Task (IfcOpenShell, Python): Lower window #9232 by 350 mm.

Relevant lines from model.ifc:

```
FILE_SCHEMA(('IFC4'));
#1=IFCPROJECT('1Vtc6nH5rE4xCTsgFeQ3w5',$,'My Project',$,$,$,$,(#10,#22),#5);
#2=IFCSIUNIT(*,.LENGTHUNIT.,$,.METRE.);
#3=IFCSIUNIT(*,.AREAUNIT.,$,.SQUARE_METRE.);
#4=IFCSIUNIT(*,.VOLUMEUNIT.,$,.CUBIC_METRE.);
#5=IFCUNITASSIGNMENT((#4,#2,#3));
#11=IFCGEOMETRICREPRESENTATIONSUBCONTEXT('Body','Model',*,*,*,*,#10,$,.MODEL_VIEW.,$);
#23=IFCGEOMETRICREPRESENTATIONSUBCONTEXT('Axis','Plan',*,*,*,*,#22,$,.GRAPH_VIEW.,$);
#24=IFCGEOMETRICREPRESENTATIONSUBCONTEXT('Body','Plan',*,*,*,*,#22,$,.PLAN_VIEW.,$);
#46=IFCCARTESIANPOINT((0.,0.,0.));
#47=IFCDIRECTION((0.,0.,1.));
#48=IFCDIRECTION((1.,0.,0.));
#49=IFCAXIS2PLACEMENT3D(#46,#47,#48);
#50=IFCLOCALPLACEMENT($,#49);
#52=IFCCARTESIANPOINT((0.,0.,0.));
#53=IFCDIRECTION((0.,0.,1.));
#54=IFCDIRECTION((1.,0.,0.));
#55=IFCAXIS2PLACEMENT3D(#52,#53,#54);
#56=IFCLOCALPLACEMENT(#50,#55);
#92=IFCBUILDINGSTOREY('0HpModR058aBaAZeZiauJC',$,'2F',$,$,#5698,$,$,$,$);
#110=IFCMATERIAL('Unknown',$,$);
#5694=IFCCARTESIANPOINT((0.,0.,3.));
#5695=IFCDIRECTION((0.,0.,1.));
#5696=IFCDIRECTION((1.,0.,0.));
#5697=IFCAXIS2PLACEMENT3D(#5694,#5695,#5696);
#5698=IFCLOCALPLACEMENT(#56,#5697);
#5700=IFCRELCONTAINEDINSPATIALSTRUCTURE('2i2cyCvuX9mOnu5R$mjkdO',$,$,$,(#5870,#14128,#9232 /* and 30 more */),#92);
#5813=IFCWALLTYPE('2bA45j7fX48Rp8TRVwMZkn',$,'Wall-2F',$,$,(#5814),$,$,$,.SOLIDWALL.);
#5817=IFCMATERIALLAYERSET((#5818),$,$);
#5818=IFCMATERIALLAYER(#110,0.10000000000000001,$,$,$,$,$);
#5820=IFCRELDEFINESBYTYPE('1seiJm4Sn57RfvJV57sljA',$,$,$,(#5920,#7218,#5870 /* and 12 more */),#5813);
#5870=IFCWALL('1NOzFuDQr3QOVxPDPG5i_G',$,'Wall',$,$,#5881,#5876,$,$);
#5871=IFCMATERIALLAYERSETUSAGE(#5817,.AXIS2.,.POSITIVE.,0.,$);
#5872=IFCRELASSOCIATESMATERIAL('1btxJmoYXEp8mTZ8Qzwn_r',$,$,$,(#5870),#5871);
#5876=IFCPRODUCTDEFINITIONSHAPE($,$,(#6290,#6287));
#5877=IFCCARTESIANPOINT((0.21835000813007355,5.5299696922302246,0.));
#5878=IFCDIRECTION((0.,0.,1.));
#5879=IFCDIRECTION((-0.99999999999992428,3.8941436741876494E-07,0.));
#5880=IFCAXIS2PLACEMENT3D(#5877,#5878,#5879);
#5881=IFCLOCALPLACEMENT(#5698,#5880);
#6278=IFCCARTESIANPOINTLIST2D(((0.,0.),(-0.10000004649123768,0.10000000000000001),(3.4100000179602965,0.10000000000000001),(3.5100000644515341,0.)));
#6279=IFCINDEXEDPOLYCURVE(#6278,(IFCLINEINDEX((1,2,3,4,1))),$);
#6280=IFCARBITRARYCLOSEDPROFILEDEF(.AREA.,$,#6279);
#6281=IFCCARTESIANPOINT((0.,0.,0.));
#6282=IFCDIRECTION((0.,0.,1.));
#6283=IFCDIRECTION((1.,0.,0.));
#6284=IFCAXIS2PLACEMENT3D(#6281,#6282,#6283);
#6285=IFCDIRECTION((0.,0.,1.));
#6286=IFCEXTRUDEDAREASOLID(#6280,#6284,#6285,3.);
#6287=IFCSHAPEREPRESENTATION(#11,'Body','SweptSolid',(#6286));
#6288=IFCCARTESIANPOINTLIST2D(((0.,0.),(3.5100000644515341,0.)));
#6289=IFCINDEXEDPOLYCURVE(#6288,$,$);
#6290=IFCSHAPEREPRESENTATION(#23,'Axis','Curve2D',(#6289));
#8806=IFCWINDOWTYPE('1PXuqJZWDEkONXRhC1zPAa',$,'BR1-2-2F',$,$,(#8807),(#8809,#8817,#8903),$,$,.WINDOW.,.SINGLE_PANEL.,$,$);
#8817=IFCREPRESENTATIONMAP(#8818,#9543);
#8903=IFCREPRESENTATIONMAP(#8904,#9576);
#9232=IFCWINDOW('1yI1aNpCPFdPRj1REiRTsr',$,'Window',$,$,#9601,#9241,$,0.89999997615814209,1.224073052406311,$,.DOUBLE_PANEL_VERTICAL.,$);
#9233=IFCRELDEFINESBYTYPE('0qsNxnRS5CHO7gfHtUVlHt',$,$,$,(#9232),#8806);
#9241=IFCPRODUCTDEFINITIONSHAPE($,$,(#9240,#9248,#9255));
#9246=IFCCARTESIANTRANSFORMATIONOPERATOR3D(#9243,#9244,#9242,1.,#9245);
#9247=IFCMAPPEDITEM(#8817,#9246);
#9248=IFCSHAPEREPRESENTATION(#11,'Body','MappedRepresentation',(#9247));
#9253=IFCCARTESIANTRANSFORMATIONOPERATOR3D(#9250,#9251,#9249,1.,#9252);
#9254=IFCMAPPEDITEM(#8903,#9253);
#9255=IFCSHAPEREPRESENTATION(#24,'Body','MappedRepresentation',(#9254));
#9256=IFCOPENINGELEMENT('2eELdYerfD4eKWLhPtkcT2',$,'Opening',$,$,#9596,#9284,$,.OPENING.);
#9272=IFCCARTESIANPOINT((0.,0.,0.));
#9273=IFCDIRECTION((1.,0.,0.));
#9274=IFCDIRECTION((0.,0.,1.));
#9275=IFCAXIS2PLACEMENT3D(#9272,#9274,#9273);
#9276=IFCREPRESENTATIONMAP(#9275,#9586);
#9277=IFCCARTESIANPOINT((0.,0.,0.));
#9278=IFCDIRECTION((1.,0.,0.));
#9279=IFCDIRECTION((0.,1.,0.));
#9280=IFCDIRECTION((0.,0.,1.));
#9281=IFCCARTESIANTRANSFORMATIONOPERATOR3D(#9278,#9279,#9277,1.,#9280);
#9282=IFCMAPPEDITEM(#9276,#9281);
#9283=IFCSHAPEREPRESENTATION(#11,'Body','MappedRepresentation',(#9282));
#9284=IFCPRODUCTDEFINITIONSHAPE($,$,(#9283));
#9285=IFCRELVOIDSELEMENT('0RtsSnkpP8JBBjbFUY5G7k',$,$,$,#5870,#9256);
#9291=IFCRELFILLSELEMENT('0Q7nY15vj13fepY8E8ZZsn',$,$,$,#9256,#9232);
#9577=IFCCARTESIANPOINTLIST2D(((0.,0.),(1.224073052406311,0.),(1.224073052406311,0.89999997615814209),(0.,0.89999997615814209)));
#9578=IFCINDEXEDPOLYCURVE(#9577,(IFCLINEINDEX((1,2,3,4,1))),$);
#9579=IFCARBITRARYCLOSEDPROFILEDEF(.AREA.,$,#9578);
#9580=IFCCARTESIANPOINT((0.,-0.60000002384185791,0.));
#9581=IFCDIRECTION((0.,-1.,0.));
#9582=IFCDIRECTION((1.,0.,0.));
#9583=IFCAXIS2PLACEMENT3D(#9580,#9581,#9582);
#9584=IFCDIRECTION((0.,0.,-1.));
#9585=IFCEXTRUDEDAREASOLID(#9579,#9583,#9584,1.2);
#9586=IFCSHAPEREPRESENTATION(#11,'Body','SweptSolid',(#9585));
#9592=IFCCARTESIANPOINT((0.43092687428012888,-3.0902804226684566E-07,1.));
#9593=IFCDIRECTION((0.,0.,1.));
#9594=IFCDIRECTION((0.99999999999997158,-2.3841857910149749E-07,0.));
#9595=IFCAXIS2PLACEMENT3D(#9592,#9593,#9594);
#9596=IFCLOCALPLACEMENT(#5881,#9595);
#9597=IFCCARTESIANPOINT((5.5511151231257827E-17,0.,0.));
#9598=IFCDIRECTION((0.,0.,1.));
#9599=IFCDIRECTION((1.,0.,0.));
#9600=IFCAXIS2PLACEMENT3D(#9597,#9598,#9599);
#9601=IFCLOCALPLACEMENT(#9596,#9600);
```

```python
import numpy as np
import ifcopenshell
import ifcopenshell.api.geometry
import ifcopenshell.util.placement
import ifcopenshell.util.unit

model = ifcopenshell.open("model.ifc")
unit_scale = ifcopenshell.util.unit.calculate_unit_scale(model)

window = model.by_id(9232)
opening = window.FillsVoids[0].RelatingOpeningElement
dz = -0.35

shift = np.array([0.0, 0.0, dz])
# The window is placed relative to its opening, so it follows when the opening moves.
matrix = ifcopenshell.util.placement.get_local_placement(opening.ObjectPlacement)
matrix[:3, 3] += shift
ifcopenshell.api.geometry.edit_object_placement(
    model, product=opening, matrix=matrix, is_si=False, should_transform_children=True
)

print(f"moved by {dz * unit_scale:+.3f} m")

model.write("model_edited.ifc")
```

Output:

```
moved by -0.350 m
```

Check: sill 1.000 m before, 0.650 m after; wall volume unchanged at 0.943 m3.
